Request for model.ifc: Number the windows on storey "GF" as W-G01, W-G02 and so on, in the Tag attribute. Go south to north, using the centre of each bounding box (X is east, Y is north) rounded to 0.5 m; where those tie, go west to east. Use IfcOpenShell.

First a look at what the model holds.

```python
import ifcopenshell
import ifcopenshell.util.element
import ifcopenshell.util.placement

model = ifcopenshell.open("model.ifc")
print(model.schema)
storey = next(s for s in model.by_type("IfcBuildingStorey") if s.Name == "GF")
windows = [e for e in ifcopenshell.util.element.get_decomposition(storey) if e.is_a("IfcWindow")]
for e in sorted(windows, key=lambda e: e.id()):
    origin = ifcopenshell.util.placement.get_local_placement(e.ObjectPlacement)[:3, 3]
    print(e.id(), e.Tag, e.Name, origin.round(2) + 0.0, sep=" | ")
```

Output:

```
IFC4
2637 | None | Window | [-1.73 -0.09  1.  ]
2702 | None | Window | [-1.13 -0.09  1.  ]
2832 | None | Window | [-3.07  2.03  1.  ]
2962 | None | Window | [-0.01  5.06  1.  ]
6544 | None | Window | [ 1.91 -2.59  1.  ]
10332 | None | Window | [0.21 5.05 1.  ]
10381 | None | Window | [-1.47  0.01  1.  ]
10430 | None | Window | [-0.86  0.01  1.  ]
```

```python
import ifcopenshell
import ifcopenshell.geom
import ifcopenshell.util.element
import ifcopenshell.util.shape

model = ifcopenshell.open("model.ifc")
settings = ifcopenshell.geom.settings()
settings.set("use-world-coords", True)


def centre(element):
    shape = ifcopenshell.geom.create_shape(settings, element)
    return ifcopenshell.util.shape.get_bbox_centroid(shape.geometry)


storey = next(s for s in model.by_type("IfcBuildingStorey") if s.Name == "GF")
windows = [e for e in ifcopenshell.util.element.get_decomposition(storey) if e.is_a("IfcWindow")]

# Insertion points can sit at a corner or the storey origin, so sort by the geometry (in metres).
centres = {e: centre(e) for e in windows}
windows.sort(key=lambda e: (round(centres[e][1] / 0.5), centres[e][0]))

for i, e in enumerate(windows, start=1):
    number = f"W-G{i:02d}"
    e.Tag = number
    print(e.id(), number)

model.write("model_rev.ifc")
```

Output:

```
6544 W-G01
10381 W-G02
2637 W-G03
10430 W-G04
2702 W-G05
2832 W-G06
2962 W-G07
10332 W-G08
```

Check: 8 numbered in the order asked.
